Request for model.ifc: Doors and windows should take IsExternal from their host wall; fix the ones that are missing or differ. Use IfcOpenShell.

First a look at what the model holds.

```python
import ifcopenshell
import ifcopenshell.util.element

model = ifcopenshell.open("model.ifc")
print(model.schema)
seen = {}
for e in model.by_type("IfcDoor") + model.by_type("IfcWindow"):
    if not e.FillsVoids:
        continue
    host = e.FillsVoids[0].RelatingOpeningElement.VoidsElements[0].RelatingBuildingElement
    own = ifcopenshell.util.element.get_pset(e, f"Pset_{e.is_a()[3:].removesuffix('StandardCase')}Common", "IsExternal")
    wall = ifcopenshell.util.element.get_pset(host, "Pset_WallCommon", "IsExternal")
    seen[e.is_a(), own, wall] = seen.get((e.is_a(), own, wall), 0) + 1
for (cls, own, wall), count in sorted(seen.items(), key=str):
    print(count, cls, "IsExternal:", own, "| host wall:", wall)
```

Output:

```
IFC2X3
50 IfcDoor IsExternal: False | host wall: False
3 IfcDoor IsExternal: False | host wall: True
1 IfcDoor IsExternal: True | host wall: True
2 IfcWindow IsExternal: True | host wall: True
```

```python
import ifcopenshell
import ifcopenshell.api.pset
import ifcopenshell.util.element

model = ifcopenshell.open("model.ifc")

count = 0
for ifc_class, pset_name in (("IfcDoor", "Pset_DoorCommon"), ("IfcWindow", "Pset_WindowCommon")):
    for e in model.by_type(ifc_class):
        if not e.FillsVoids:
            continue
        host = e.FillsVoids[0].RelatingOpeningElement.VoidsElements[0].RelatingBuildingElement
        external = ifcopenshell.util.element.get_pset(host, "Pset_WallCommon", "IsExternal")
        if external is None or ifcopenshell.util.element.get_pset(e, pset_name, "IsExternal") == external:
            continue
        pset = ifcopenshell.api.pset.add_pset(model, product=e, name=pset_name)
        ifcopenshell.api.pset.edit_pset(model, pset=pset, properties={"IsExternal": external})
        count += 1

print(count, "updated")

model.write("model_rev.ifc")
```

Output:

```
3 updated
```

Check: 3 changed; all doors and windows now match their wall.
